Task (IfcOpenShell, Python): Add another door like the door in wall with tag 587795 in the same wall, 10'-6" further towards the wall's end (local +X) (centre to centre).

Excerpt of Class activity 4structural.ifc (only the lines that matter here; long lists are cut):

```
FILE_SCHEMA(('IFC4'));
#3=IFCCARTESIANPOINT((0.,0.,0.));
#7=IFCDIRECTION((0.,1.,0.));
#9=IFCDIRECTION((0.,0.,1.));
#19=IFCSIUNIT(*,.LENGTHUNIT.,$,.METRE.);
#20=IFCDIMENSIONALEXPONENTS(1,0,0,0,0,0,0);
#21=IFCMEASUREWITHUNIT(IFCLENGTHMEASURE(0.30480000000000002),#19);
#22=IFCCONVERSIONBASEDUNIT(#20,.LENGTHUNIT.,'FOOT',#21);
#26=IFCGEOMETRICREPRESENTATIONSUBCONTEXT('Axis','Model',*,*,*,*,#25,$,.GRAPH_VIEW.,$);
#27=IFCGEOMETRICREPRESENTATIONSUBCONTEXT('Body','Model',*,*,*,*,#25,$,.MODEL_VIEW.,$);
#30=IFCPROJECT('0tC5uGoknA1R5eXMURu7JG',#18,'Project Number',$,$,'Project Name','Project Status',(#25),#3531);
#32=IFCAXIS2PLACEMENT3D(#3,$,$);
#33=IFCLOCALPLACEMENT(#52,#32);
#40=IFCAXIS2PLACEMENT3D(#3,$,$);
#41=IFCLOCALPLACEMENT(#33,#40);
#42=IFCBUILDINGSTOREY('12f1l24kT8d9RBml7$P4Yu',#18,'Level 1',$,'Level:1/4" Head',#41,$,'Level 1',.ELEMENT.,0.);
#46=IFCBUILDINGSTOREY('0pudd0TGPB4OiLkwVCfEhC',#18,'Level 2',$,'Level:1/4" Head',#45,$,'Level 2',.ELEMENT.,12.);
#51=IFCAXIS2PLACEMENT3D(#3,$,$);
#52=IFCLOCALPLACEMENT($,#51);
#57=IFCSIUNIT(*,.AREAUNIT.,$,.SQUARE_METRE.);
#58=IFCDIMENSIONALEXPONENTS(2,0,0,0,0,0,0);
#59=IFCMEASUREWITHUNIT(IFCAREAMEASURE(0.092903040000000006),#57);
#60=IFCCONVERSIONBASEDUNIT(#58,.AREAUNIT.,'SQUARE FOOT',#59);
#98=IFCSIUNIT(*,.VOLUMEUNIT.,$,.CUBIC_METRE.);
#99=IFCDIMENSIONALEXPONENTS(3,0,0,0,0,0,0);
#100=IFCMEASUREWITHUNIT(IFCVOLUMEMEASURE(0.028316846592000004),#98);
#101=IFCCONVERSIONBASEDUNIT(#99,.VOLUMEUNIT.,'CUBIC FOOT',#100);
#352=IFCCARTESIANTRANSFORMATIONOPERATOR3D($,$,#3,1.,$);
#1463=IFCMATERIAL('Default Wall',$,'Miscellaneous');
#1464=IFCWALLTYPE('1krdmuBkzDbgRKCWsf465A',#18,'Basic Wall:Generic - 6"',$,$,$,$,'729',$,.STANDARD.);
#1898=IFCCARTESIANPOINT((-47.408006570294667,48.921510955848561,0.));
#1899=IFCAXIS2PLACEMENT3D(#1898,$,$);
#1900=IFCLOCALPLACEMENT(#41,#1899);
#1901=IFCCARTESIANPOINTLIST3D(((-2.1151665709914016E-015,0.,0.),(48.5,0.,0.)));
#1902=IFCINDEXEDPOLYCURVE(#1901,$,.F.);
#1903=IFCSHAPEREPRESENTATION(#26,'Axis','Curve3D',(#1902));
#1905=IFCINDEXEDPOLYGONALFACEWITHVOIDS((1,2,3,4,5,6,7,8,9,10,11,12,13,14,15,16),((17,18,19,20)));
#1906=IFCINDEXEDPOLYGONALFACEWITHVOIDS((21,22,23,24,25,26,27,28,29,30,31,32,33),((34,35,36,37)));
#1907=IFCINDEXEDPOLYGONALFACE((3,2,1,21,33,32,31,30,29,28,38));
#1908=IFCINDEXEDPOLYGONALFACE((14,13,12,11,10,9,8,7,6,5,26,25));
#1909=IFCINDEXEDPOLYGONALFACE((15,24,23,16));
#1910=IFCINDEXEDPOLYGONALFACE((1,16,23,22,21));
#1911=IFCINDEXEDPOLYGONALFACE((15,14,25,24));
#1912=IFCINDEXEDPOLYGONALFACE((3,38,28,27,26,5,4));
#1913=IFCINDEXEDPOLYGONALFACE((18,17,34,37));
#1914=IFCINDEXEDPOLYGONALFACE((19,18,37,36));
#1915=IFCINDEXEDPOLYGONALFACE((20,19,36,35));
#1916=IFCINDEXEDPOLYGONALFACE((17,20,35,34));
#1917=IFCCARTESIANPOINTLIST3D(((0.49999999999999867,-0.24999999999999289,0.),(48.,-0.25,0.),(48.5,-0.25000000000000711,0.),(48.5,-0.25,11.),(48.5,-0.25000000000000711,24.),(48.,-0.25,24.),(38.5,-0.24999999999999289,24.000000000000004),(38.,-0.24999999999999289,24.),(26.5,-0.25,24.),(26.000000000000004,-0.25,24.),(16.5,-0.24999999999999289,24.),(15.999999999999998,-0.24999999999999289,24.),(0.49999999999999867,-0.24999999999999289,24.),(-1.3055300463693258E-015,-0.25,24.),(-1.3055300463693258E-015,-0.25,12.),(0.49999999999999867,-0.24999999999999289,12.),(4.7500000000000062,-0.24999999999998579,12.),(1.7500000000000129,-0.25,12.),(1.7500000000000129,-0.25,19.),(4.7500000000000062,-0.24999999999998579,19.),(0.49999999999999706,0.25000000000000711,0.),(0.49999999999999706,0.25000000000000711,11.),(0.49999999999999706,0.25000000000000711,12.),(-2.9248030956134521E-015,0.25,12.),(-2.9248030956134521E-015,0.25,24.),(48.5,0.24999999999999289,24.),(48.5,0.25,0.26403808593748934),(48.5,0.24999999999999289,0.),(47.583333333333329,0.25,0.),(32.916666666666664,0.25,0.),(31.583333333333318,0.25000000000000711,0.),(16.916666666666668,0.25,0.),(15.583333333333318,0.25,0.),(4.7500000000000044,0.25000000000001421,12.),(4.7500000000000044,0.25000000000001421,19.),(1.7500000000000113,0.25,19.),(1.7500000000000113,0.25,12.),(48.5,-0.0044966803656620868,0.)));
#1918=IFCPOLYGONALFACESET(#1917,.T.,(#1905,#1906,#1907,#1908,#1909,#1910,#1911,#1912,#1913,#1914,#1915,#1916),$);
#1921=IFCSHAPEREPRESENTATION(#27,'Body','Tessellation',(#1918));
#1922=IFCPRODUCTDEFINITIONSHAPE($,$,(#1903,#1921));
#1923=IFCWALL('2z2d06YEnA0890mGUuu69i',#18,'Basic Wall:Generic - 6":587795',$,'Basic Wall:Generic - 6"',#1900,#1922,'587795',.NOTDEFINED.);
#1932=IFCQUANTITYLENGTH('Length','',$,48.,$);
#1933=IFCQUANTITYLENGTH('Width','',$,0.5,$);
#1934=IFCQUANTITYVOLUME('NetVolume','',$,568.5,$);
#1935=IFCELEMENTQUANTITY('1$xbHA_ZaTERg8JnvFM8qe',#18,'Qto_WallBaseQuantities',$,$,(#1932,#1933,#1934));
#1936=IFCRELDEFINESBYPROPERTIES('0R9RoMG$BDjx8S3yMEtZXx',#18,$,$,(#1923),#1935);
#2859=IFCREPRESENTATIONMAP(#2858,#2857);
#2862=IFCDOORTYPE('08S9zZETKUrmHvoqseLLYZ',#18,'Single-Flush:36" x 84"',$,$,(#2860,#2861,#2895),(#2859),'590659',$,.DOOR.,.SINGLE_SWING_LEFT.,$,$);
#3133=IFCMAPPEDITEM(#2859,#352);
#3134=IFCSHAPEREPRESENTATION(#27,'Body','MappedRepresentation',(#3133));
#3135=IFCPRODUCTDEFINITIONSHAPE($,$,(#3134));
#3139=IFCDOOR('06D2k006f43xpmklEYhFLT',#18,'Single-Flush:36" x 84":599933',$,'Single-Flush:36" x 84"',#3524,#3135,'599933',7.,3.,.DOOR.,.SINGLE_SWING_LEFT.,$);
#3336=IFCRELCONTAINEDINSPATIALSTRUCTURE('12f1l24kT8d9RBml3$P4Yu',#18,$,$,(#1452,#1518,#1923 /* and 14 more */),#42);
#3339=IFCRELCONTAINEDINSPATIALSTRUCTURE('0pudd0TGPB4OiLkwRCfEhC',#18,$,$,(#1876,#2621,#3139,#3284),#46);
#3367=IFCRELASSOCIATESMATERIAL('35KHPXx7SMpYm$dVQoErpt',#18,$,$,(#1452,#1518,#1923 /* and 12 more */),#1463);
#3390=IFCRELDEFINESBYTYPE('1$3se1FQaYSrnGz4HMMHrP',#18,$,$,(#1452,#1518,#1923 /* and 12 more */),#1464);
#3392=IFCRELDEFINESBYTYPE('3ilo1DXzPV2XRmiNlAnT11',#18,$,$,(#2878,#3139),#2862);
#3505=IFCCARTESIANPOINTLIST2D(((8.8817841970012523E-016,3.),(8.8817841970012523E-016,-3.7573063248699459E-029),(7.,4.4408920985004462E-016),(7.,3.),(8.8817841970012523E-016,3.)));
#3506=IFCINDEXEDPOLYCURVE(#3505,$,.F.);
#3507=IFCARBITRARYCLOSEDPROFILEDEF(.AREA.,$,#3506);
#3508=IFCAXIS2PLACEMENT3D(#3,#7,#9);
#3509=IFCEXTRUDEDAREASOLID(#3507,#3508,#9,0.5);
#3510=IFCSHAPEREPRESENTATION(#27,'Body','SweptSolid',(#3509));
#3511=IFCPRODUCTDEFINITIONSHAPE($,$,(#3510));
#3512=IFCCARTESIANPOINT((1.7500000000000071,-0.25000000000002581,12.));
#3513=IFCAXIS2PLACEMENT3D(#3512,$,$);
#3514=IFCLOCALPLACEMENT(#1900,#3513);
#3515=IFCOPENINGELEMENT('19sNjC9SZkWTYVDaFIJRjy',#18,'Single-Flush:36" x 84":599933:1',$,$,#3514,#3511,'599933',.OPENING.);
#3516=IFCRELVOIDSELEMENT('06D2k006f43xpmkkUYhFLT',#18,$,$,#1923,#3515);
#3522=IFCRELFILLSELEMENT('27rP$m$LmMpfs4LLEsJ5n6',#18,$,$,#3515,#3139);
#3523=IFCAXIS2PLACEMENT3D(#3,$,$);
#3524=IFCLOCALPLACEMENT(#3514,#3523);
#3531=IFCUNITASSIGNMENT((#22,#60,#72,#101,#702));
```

```python
import ifcopenshell
import ifcopenshell.api.feature
import ifcopenshell.api.geometry
import ifcopenshell.api.pset
import ifcopenshell.api.root
import ifcopenshell.geom
import ifcopenshell.util.element
import ifcopenshell.util.placement
import ifcopenshell.util.shape
import ifcopenshell.util.unit

model = ifcopenshell.open("Class activity 4structural.ifc")
unit_scale = ifcopenshell.util.unit.calculate_unit_scale(model)
volume_scale = ifcopenshell.util.unit.calculate_unit_scale(model, "VOLUMEUNIT")
settings = ifcopenshell.geom.settings()


def volume(element):
    """Net volume in cubic metres, openings subtracted."""
    shape = ifcopenshell.geom.create_shape(settings, element)
    return ifcopenshell.util.shape.get_volume(shape.geometry)


def reuse_history(source, copy):
    """copy_class also copies each property set's owner history, people and application; keep the originals."""
    for rel in copy.IsDefinedBy:
        if rel.is_a("IfcRelDefinesByProperties") and (history := rel.RelatingPropertyDefinition.OwnerHistory):
            rel.RelatingPropertyDefinition.OwnerHistory = source.OwnerHistory
            ifcopenshell.util.element.remove_deep2(model, history)


door = model.by_id(3139)
opening = door.FillsVoids[0].RelatingOpeningElement
wall = opening.VoidsElements[0].RelatingBuildingElement
before = volume(wall)
shift = ifcopenshell.util.placement.get_local_placement(wall.ObjectPlacement)[:3, 0] * 126 * 0.0254 / unit_scale

# copy_class copies the void relationship, type, container and properties, but no geometry.
new_opening = ifcopenshell.api.root.copy_class(model, product=opening)
new_opening.Representation = ifcopenshell.util.element.copy_deep(
    model, opening.Representation, exclude=["IfcGeometricRepresentationContext", "IfcRepresentationMap"]
)
new_opening.Name = 'Single-Flush:36" x 84"'
new_opening.Tag = None
reuse_history(opening, new_opening)
new_door = ifcopenshell.api.root.copy_class(model, product=door)
new_door.Representation = ifcopenshell.util.element.copy_deep(
    model, door.Representation, exclude=["IfcGeometricRepresentationContext", "IfcRepresentationMap"]
)
new_door.Name = 'Single-Flush:36" x 84"'
new_door.Tag = None
reuse_history(door, new_door)
ifcopenshell.api.feature.add_filling(model, opening=new_opening, element=new_door)

for old, new in ((opening, new_opening), (door, new_door)):
    matrix = ifcopenshell.util.placement.get_local_placement(old.ObjectPlacement)
    matrix[:3, 3] += shift
    ifcopenshell.api.geometry.edit_object_placement(model, product=new, matrix=matrix, is_si=False)

after = volume(wall)

# Update the wall's stored quantities.
qto = model.by_id(ifcopenshell.util.element.get_pset(wall, "Qto_WallBaseQuantities", should_inherit=False)["id"])
ifcopenshell.api.pset.edit_qto(model, qto=qto, properties={"NetVolume": after / volume_scale})

print(f"wall volume {before:.3f} -> {after:.3f} m3")

model.write("Class activity 4structural_rev.ifc")
```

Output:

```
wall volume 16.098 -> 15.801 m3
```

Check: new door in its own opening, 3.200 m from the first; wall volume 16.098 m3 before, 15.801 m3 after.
